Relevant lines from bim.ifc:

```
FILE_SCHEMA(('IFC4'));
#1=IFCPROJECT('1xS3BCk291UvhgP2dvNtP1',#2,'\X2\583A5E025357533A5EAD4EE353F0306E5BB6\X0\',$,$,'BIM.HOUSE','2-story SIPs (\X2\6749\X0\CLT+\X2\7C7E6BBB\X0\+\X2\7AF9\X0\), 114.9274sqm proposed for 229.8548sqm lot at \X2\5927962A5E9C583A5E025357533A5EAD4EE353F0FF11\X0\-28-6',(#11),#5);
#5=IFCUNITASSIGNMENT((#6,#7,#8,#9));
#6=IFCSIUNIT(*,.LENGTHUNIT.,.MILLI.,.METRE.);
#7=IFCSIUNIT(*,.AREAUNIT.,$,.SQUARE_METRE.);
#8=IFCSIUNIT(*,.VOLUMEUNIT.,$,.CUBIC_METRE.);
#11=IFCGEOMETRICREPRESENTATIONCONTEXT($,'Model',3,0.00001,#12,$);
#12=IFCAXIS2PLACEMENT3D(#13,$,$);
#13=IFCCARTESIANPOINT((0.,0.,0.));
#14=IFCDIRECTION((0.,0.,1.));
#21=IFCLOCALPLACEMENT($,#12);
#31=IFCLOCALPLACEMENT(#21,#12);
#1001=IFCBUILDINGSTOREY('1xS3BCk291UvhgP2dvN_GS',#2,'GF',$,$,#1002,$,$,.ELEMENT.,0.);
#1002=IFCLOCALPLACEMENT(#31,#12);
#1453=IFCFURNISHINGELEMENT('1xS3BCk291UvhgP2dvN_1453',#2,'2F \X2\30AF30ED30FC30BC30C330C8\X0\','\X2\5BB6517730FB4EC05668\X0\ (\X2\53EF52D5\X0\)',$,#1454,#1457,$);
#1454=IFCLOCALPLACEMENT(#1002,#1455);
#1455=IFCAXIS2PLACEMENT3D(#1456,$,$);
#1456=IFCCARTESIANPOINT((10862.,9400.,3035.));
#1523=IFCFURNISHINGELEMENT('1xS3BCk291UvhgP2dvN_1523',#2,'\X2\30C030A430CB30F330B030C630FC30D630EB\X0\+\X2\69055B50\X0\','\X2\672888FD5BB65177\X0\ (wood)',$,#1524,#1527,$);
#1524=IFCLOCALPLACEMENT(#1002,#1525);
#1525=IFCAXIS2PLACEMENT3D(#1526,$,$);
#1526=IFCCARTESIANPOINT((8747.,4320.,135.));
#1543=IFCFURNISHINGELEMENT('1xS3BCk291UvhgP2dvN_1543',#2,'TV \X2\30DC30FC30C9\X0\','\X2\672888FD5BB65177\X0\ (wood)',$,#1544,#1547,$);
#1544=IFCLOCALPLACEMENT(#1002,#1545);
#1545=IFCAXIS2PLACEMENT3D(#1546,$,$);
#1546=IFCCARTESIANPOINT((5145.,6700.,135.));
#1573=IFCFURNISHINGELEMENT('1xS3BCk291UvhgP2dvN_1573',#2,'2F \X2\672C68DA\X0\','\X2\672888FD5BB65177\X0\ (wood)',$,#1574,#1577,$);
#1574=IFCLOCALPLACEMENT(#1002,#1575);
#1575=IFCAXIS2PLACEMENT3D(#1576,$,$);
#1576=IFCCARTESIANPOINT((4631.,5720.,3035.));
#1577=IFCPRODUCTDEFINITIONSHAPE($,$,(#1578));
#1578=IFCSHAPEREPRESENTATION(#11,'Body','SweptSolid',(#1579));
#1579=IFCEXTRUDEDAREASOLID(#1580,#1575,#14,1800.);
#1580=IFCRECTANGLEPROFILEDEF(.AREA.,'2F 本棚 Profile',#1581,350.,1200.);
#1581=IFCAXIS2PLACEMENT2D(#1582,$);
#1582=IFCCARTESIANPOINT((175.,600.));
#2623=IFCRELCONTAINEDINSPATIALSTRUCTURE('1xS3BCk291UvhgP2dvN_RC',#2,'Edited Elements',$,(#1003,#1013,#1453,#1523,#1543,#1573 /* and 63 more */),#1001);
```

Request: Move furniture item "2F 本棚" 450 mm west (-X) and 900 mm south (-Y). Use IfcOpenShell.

```python
import ifcopenshell
import ifcopenshell.api.geometry
import ifcopenshell.util.placement

model = ifcopenshell.open("bim.ifc")

item = model.by_guid("1xS3BCk291UvhgP2dvN_1573")
matrix = ifcopenshell.util.placement.get_local_placement(item.ObjectPlacement)
matrix[0, 3] -= 450.0
matrix[1, 3] -= 900.0
ifcopenshell.api.geometry.edit_object_placement(model, product=item, matrix=matrix, is_si=False)

print(ifcopenshell.util.placement.get_local_placement(item.ObjectPlacement).round(3) + 0.0)

model.write("bim_rev.ifc")
```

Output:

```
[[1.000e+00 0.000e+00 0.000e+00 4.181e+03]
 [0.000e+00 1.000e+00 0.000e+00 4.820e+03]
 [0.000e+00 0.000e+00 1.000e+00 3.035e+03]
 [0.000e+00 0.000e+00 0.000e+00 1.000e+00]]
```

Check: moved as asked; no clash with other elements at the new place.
